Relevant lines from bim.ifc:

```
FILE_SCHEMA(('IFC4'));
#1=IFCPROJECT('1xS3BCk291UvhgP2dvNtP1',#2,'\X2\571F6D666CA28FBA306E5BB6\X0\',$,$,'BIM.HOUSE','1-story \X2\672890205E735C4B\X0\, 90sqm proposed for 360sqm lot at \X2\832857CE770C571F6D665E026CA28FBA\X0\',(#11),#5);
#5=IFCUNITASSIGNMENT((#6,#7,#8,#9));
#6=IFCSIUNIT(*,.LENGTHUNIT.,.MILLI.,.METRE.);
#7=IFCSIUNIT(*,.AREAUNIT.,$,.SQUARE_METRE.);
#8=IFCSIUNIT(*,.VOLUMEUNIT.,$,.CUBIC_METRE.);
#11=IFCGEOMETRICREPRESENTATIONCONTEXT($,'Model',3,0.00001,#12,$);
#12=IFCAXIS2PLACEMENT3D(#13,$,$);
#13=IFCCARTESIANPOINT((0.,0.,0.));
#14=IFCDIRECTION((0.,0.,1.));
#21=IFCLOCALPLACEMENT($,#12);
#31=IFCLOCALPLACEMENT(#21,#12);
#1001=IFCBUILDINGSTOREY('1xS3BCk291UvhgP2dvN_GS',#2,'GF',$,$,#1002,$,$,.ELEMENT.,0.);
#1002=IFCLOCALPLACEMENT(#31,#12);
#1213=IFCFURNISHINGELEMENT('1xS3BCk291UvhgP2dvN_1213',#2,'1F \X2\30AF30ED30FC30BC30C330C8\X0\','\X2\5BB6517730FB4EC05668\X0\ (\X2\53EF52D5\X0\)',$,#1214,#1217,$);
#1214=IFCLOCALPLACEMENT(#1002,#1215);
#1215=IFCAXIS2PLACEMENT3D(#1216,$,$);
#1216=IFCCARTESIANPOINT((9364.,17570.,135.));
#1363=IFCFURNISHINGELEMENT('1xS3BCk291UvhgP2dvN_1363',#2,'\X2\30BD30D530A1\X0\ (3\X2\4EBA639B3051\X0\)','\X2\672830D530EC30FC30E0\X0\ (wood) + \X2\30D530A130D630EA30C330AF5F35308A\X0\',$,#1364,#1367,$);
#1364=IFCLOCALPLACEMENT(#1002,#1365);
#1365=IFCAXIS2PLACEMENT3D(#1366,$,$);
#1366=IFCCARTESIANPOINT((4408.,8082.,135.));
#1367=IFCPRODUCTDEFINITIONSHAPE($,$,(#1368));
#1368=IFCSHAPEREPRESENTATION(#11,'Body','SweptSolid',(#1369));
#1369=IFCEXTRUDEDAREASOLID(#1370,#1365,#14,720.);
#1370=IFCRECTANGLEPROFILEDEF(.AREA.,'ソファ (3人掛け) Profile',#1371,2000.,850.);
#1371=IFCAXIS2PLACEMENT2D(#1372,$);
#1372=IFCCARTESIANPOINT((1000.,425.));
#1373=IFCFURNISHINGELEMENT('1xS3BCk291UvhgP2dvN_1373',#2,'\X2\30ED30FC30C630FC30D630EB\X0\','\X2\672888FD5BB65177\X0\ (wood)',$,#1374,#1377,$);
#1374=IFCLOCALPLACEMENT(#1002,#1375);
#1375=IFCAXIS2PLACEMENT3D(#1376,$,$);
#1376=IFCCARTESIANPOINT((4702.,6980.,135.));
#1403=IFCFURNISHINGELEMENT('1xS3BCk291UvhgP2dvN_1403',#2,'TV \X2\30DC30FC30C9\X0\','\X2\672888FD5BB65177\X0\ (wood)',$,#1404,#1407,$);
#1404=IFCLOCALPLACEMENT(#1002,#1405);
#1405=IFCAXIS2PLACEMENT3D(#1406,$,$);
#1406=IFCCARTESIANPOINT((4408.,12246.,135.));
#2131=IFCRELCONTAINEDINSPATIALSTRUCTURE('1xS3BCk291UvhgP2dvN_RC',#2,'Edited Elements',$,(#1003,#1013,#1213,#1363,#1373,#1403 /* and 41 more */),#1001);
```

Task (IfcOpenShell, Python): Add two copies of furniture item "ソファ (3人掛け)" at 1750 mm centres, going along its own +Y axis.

```python
import ifcopenshell
import ifcopenshell.api.geometry
import ifcopenshell.api.root
import ifcopenshell.util.element
import ifcopenshell.util.placement

model = ifcopenshell.open("bim.ifc")


def reuse_history(source, copy):
    """copy_class also copies each property set's owner history, people and application; keep the originals."""
    for rel in copy.IsDefinedBy:
        if rel.is_a("IfcRelDefinesByProperties") and (history := rel.RelatingPropertyDefinition.OwnerHistory):
            rel.RelatingPropertyDefinition.OwnerHistory = source.OwnerHistory
            ifcopenshell.util.element.remove_deep2(model, history)


source = model.by_guid("1xS3BCk291UvhgP2dvN_1363")
base = ifcopenshell.util.placement.get_local_placement(source.ObjectPlacement)
step = base[:3, 1] * 1750.0

for i in range(1, 3):
    copy = ifcopenshell.api.root.copy_class(model, product=source)
    copy.Representation = ifcopenshell.util.element.copy_deep(
        model, source.Representation, exclude=["IfcGeometricRepresentationContext", "IfcRepresentationMap"]
    )
    reuse_history(source, copy)
    matrix = base.copy()
    matrix[:3, 3] += i * step
    print("added at", matrix[:3, 3].round(3) + 0.0)
    ifcopenshell.api.geometry.edit_object_placement(model, product=copy, matrix=matrix, is_si=False)

model.write("bim_v2.ifc")
```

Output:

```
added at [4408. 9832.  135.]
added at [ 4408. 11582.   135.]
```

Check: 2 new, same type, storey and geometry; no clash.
